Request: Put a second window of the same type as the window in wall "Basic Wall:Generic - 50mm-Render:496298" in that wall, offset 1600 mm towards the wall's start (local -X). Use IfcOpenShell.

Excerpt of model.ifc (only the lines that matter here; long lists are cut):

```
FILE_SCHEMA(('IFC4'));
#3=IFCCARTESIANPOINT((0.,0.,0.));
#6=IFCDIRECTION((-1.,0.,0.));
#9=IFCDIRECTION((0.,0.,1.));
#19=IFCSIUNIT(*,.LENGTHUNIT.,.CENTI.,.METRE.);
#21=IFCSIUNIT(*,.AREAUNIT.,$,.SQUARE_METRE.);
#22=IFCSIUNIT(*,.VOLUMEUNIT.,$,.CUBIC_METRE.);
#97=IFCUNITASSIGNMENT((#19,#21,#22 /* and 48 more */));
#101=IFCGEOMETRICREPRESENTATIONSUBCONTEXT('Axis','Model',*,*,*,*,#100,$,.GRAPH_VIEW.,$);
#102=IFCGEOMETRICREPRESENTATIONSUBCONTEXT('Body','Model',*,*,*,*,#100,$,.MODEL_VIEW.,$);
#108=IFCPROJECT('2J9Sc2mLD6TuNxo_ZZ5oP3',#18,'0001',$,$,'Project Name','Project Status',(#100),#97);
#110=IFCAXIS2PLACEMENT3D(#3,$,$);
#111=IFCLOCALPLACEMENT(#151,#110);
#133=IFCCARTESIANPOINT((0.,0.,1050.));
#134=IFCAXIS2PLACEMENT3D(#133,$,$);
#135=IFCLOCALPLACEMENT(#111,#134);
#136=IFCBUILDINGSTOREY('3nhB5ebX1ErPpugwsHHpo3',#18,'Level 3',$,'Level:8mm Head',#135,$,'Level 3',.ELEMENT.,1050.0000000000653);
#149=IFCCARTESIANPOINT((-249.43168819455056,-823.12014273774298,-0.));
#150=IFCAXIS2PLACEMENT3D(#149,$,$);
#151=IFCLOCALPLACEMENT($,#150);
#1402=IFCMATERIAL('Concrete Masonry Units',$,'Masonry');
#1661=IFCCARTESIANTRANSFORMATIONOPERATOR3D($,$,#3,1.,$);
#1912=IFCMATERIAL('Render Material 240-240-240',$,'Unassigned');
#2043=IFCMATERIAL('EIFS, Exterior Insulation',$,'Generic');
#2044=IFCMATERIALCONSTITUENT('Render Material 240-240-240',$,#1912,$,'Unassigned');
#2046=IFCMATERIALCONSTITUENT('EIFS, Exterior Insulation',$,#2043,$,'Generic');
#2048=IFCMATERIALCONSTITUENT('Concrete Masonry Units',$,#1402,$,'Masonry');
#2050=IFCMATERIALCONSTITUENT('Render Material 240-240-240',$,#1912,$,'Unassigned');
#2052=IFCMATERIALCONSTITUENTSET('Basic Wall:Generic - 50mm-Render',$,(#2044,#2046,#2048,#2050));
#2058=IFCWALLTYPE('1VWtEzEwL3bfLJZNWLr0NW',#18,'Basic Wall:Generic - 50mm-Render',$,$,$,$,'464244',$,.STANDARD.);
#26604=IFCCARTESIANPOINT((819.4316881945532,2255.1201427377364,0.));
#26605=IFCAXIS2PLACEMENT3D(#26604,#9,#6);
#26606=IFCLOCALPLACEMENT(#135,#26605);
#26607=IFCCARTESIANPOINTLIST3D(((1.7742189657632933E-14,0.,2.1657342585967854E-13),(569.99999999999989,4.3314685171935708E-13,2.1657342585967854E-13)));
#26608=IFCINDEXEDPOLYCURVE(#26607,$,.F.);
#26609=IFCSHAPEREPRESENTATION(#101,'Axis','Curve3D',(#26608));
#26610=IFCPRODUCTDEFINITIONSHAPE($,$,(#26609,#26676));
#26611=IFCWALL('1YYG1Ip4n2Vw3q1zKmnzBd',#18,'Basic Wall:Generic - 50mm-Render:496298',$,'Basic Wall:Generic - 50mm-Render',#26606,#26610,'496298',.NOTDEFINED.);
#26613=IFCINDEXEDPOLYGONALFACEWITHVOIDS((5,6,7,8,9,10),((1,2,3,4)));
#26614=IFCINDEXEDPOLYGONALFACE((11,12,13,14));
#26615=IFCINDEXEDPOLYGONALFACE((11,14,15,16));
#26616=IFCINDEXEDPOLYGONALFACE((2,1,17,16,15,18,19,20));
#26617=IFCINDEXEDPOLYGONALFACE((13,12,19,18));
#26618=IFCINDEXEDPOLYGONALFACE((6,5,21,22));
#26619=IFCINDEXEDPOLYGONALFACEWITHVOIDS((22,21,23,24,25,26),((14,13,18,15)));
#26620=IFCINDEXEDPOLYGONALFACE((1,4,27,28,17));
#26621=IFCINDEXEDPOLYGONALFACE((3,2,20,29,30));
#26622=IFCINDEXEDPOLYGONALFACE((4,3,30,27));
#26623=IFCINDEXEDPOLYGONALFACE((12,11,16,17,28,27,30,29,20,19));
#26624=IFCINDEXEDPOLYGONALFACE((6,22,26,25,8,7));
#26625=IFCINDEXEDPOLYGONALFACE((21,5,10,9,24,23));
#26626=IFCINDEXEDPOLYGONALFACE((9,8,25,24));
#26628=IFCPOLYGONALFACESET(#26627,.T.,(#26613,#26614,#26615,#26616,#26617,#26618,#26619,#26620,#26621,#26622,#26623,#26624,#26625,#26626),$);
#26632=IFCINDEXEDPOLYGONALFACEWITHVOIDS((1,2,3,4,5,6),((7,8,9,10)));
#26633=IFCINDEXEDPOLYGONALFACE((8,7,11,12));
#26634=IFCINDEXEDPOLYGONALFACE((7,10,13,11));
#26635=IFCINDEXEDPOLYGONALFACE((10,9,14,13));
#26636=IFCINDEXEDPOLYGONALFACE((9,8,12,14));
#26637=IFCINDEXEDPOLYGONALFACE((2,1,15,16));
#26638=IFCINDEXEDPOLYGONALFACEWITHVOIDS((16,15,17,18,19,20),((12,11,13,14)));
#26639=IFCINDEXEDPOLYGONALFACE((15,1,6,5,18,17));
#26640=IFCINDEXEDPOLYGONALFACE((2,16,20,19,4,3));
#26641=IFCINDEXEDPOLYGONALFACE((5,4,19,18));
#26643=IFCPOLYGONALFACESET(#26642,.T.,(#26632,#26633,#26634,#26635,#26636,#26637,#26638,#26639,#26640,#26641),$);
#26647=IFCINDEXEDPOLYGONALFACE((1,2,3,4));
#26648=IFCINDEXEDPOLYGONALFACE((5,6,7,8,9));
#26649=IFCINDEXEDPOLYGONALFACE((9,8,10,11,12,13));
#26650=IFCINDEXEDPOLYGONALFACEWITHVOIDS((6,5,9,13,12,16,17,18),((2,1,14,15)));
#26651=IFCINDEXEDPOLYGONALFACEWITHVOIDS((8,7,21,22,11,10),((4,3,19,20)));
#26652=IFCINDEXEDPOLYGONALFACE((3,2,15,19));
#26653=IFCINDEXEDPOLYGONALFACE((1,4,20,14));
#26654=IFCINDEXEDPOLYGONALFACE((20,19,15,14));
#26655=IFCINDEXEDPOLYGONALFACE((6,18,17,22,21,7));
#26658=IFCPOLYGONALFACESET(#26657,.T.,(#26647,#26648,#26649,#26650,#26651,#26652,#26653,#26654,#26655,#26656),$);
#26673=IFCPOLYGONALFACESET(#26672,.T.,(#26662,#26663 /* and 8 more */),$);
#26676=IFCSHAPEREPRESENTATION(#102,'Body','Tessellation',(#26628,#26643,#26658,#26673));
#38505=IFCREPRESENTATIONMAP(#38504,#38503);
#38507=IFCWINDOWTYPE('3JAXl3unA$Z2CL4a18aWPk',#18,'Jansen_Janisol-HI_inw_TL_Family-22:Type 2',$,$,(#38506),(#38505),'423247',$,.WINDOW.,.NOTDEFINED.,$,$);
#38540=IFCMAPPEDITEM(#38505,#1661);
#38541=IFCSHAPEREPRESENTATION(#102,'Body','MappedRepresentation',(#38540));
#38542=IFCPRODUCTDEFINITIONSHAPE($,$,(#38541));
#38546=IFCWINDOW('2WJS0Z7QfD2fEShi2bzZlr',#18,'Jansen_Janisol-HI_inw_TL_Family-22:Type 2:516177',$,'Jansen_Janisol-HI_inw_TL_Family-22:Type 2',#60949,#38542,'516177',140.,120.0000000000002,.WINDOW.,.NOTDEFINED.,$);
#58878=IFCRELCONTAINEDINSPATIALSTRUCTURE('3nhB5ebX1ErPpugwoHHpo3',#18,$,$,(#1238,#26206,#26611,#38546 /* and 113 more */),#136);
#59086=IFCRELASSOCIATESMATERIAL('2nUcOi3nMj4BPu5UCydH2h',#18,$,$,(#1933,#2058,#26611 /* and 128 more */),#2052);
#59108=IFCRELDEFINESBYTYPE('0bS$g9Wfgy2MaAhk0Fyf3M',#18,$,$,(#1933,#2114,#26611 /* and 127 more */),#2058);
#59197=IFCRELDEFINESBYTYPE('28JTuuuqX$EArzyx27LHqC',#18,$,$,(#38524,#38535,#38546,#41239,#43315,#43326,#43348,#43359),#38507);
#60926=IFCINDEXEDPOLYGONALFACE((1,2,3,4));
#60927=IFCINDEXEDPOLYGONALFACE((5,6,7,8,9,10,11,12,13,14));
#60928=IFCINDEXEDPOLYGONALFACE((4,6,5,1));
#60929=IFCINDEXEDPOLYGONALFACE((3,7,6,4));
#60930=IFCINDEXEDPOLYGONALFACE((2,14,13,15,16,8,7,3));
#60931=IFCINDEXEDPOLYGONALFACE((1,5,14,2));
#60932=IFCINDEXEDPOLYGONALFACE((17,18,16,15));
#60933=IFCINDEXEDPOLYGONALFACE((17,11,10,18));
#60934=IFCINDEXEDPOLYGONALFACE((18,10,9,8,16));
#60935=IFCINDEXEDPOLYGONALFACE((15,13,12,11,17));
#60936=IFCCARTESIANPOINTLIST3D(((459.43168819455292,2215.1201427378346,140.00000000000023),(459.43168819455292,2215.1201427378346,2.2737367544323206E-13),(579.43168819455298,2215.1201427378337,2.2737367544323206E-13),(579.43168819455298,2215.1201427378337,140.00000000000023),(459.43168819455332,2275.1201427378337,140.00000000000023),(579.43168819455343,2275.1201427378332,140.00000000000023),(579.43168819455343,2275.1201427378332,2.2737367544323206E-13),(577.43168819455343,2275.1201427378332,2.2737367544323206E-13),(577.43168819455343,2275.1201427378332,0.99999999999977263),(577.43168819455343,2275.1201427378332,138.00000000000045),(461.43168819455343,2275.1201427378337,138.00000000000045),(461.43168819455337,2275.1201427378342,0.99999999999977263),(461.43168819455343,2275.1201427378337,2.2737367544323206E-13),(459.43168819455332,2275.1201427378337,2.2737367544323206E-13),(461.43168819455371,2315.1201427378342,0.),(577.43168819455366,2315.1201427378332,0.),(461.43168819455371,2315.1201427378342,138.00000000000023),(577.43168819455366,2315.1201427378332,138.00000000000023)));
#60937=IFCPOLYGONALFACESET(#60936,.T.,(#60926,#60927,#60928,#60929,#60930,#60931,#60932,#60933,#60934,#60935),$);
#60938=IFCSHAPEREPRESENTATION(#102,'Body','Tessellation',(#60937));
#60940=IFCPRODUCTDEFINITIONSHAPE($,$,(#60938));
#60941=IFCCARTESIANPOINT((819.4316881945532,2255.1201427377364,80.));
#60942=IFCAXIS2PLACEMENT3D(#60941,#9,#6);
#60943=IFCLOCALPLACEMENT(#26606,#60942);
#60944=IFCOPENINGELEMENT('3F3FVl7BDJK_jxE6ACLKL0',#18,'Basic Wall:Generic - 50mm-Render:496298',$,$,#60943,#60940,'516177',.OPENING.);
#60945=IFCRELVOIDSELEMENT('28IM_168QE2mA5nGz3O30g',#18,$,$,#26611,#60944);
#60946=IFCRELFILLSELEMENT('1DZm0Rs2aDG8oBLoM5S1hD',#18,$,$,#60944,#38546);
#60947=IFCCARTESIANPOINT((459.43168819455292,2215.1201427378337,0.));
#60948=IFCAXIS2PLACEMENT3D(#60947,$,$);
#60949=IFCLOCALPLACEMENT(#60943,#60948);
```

```python
import ifcopenshell
import ifcopenshell.api.feature
import ifcopenshell.api.geometry
import ifcopenshell.api.root
import ifcopenshell.geom
import ifcopenshell.util.element
import ifcopenshell.util.placement
import ifcopenshell.util.shape
import ifcopenshell.util.unit

model = ifcopenshell.open("model.ifc")
unit_scale = ifcopenshell.util.unit.calculate_unit_scale(model)
settings = ifcopenshell.geom.settings()


def volume(element):
    """Net volume in cubic metres, openings subtracted."""
    shape = ifcopenshell.geom.create_shape(settings, element)
    return ifcopenshell.util.shape.get_volume(shape.geometry)


window = model.by_guid("2WJS0Z7QfD2fEShi2bzZlr")
opening = window.FillsVoids[0].RelatingOpeningElement
wall = opening.VoidsElements[0].RelatingBuildingElement
before = volume(wall)
shift = ifcopenshell.util.placement.get_local_placement(wall.ObjectPlacement)[:3, 0] * -1.6 / unit_scale

# copy_class copies the void relationship, type, container and properties, but no geometry.
new_opening = ifcopenshell.api.root.copy_class(model, product=opening)
new_opening.Representation = ifcopenshell.util.element.copy_deep(
    model, opening.Representation, exclude=["IfcGeometricRepresentationContext", "IfcRepresentationMap"]
)
new_opening.Name = "Basic Wall:Generic - 50mm-Render"
new_opening.Tag = None
new_window = ifcopenshell.api.root.copy_class(model, product=window)
new_window.Representation = ifcopenshell.util.element.copy_deep(
    model, window.Representation, exclude=["IfcGeometricRepresentationContext", "IfcRepresentationMap"]
)
new_window.Name = "Jansen_Janisol-HI_inw_TL_Family-22:Type 2"
new_window.Tag = None
ifcopenshell.api.feature.add_filling(model, opening=new_opening, element=new_window)

for old, new in ((opening, new_opening), (window, new_window)):
    matrix = ifcopenshell.util.placement.get_local_placement(old.ObjectPlacement)
    matrix[:3, 3] += shift
    ifcopenshell.api.geometry.edit_object_placement(model, product=new, matrix=matrix, is_si=False)

after = volume(wall)

print(f"wall volume {before:.3f} -> {after:.3f} m3")

model.write("model-out.ifc")
```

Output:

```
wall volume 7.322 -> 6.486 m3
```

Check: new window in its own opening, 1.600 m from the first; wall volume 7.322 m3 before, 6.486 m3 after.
